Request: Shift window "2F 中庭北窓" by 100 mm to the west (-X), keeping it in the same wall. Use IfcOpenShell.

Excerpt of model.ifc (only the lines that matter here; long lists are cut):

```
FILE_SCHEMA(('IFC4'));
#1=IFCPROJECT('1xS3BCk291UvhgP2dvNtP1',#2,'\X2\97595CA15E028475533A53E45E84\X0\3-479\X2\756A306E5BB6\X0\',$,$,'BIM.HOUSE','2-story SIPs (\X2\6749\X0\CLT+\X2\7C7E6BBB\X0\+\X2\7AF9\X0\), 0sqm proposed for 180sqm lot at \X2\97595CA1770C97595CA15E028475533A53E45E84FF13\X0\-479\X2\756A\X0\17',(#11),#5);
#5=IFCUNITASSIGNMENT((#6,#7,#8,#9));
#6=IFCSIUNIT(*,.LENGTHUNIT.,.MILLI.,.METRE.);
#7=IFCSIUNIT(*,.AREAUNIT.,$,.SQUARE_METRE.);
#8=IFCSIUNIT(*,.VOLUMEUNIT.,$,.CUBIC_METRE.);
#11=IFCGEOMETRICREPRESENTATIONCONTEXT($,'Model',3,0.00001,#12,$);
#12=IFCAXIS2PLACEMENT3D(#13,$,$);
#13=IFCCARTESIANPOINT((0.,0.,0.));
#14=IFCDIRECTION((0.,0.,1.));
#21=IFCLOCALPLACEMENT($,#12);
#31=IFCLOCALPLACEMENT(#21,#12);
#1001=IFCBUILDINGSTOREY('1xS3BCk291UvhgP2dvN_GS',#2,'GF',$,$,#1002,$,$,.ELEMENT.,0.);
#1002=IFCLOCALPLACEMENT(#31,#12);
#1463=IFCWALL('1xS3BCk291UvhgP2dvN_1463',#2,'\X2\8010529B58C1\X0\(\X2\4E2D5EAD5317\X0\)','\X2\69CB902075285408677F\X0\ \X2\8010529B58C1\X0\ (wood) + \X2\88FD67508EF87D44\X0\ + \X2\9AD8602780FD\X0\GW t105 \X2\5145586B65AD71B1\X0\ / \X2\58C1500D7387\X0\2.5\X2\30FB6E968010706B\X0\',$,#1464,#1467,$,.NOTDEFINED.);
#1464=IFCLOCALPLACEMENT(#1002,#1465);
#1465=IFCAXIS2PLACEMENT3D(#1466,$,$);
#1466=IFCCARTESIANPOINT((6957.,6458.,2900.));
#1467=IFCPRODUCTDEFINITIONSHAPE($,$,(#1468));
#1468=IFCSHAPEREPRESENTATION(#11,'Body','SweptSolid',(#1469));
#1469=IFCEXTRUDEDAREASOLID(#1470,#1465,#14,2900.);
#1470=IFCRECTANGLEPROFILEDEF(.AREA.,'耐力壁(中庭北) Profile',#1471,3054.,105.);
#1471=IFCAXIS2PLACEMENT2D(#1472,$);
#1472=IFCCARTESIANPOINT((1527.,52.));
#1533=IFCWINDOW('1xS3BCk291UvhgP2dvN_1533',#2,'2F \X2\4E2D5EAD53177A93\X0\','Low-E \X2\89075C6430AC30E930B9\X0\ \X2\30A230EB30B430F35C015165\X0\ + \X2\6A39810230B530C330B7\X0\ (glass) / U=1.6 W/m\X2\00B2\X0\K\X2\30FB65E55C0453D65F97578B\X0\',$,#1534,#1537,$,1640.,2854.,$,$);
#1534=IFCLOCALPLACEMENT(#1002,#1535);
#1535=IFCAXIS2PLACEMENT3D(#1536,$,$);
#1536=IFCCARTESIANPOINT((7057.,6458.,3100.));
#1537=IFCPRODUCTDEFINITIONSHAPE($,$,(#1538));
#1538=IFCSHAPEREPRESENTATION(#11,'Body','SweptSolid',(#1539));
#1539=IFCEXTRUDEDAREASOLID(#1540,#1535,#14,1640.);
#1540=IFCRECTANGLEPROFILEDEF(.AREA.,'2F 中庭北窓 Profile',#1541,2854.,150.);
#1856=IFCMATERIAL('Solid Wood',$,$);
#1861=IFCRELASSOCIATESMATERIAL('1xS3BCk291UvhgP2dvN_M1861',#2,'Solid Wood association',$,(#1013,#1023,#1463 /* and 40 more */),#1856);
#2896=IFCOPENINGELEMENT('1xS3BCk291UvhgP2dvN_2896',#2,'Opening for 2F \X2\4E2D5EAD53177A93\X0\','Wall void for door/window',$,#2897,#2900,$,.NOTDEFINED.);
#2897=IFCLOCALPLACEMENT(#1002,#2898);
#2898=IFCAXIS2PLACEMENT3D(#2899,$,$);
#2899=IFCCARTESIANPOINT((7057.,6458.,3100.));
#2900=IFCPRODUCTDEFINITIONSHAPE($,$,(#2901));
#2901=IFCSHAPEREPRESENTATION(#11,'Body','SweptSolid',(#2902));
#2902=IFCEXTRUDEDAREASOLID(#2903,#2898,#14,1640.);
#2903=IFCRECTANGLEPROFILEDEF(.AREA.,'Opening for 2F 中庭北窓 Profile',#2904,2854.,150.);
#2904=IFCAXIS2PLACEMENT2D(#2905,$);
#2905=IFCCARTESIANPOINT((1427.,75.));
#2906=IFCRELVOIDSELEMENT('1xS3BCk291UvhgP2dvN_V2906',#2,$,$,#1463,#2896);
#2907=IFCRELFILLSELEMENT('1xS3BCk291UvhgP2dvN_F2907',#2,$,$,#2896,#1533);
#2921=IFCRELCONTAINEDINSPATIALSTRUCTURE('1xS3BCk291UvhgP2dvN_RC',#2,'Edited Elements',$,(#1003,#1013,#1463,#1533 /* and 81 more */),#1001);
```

```python
import ifcopenshell
import ifcopenshell.api.geometry
import ifcopenshell.util.placement

model = ifcopenshell.open("model.ifc")

window = model.by_guid("1xS3BCk291UvhgP2dvN_1533")
opening = window.FillsVoids[0].RelatingOpeningElement
wall = opening.VoidsElements[0].RelatingBuildingElement

wall_matrix = ifcopenshell.util.placement.get_local_placement(wall.ObjectPlacement)
shift = wall_matrix[:3, 0] * -100.0
before = ifcopenshell.util.placement.get_local_placement(window.ObjectPlacement)[:3, 3].copy()

# The window is not placed relative to its opening, so move both.
for product in (opening, window):
    matrix = ifcopenshell.util.placement.get_local_placement(product.ObjectPlacement)
    matrix[:3, 3] += shift
    ifcopenshell.api.geometry.edit_object_placement(model, product=product, matrix=matrix, is_si=False)

after = ifcopenshell.util.placement.get_local_placement(window.ObjectPlacement)[:3, 3]
print("window moved by", (after - before).round(3) + 0.0)

model.write("model-out.ifc")
```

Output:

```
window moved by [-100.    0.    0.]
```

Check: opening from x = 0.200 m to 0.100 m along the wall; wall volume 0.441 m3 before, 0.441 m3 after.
